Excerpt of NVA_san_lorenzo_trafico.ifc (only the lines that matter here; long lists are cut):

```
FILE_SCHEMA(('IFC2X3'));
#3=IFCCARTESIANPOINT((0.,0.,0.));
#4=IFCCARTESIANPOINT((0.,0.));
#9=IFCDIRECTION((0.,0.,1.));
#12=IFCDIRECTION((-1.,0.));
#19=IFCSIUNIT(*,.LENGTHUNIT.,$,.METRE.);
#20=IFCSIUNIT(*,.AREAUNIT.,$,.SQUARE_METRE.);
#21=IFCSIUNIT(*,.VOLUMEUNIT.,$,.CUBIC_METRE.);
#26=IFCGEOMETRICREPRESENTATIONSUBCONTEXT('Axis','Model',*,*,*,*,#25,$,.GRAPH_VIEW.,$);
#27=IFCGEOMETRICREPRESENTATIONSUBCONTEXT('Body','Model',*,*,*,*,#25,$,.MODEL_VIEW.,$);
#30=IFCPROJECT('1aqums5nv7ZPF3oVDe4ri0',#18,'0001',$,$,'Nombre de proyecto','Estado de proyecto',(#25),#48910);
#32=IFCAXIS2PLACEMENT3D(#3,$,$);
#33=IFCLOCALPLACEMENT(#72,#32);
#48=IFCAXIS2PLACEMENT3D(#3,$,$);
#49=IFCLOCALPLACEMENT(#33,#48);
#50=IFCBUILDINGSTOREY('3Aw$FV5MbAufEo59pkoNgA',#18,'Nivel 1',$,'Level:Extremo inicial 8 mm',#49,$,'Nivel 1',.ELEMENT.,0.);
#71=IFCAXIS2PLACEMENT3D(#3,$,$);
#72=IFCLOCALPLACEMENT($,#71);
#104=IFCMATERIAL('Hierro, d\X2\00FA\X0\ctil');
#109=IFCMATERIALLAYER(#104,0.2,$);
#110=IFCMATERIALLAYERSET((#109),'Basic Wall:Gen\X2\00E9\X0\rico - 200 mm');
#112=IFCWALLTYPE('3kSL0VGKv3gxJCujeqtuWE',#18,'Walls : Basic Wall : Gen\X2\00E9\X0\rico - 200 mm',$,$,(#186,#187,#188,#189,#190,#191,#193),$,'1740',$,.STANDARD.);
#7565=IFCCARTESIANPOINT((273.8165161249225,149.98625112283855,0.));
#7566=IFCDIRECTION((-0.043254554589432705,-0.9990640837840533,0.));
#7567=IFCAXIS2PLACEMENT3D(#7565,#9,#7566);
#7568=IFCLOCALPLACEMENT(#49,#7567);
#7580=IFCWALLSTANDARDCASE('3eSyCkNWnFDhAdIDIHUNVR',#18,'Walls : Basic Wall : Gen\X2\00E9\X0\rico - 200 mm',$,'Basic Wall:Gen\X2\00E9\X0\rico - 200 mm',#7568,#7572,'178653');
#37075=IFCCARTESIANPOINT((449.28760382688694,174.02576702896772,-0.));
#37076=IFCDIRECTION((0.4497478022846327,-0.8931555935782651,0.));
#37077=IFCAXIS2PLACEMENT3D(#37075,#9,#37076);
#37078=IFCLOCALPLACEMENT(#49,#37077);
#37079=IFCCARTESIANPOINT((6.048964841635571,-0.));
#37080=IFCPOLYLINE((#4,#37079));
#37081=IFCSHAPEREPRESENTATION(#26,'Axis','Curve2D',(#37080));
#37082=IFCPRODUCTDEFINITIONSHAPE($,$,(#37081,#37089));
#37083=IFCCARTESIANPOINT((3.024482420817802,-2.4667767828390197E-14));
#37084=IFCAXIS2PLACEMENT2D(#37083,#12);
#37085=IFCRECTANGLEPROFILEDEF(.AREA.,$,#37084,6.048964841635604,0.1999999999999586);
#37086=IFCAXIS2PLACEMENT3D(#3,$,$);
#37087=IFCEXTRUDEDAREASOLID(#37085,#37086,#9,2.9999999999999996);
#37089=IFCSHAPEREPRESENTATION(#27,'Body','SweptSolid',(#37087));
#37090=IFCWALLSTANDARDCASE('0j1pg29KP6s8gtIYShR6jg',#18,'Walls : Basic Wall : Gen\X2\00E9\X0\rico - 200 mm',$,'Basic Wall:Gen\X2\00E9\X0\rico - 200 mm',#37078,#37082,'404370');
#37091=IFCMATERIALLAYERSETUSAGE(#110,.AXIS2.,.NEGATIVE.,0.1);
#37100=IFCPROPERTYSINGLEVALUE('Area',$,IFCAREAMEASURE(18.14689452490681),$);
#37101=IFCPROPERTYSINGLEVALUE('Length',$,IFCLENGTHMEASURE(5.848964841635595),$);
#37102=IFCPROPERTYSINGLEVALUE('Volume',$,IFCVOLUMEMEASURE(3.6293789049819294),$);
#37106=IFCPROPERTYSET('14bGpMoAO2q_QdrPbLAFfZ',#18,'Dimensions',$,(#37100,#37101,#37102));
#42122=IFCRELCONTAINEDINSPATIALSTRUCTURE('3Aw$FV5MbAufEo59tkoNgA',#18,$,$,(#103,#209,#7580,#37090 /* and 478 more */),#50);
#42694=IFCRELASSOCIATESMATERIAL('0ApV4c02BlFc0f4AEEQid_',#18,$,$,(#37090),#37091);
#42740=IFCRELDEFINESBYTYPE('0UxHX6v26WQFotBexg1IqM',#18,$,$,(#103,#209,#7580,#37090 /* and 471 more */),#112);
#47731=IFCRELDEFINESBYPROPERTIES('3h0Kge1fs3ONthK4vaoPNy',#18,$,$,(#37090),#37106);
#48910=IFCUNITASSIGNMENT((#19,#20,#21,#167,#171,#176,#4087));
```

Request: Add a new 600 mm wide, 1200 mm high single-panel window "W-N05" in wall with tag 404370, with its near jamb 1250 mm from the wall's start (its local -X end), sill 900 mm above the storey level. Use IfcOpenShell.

```python
import numpy as np
import ifcopenshell
import ifcopenshell.api.feature
import ifcopenshell.api.geometry
import ifcopenshell.api.pset
import ifcopenshell.api.root
import ifcopenshell.api.spatial
import ifcopenshell.api.type
import ifcopenshell.geom
import ifcopenshell.util.element
import ifcopenshell.util.placement
import ifcopenshell.util.representation
import ifcopenshell.util.shape
import ifcopenshell.util.unit

model = ifcopenshell.open("NVA_san_lorenzo_trafico.ifc")
unit_scale = ifcopenshell.util.unit.calculate_unit_scale(model)
area_scale = ifcopenshell.util.unit.calculate_unit_scale(model, "AREAUNIT")
volume_scale = ifcopenshell.util.unit.calculate_unit_scale(model, "VOLUMEUNIT")
settings = ifcopenshell.geom.settings()


def volume(element):
    """Net volume in cubic metres, openings subtracted."""
    shape = ifcopenshell.geom.create_shape(settings, element)
    return ifcopenshell.util.shape.get_volume(shape.geometry)


wall = model.by_guid("0j1pg29KP6s8gtIYShR6jg")
storey = ifcopenshell.util.element.get_container(wall, ifc_class="IfcBuildingStorey")
context = ifcopenshell.util.representation.get_context(model, "Model", "Body", "MODEL_VIEW")
before = volume(wall)

width, height, from_end, sill = 0.6, 1.2, 1.25, 0.9  # metres

# The wall runs along its own X axis, and the end named is its -X end.
wall_shape = ifcopenshell.geom.create_shape(settings, wall)
x, y, z = ifcopenshell.util.shape.get_vertices(wall_shape.geometry).T
start = x.min() + from_end
face, thickness = float(y.min()), float(y.max() - y.min())
wall_matrix = ifcopenshell.util.placement.get_local_placement(wall.ObjectPlacement)
level = ifcopenshell.util.placement.get_local_placement(storey.ObjectPlacement)[2, 3]


def in_wall(x, y):
    """Placement at x, y metres in the wall's axes, at sill height."""
    matrix = wall_matrix.copy()
    matrix[:, 3] = wall_matrix @ np.array([x / unit_scale, y / unit_scale, 0.0, 1.0])
    matrix[2, 3] = level + sill / unit_scale
    return matrix


# Opening: a box that overshoots both wall faces by 50 mm.
opening = ifcopenshell.api.root.create_entity(model, ifc_class="IfcOpeningElement")
box = ifcopenshell.api.geometry.add_wall_representation(
    model, context=context, length=width, height=height, thickness=thickness + 0.1
)
ifcopenshell.api.geometry.assign_representation(model, product=opening, representation=box)
ifcopenshell.api.geometry.edit_object_placement(model, product=opening, matrix=in_wall(start, face - 0.05), is_si=False)
ifcopenshell.api.feature.add_feature(model, feature=opening, element=wall)

window = ifcopenshell.api.root.create_entity(model, ifc_class="IfcWindow", name="W-N05")
window.OverallWidth, window.OverallHeight = width / unit_scale, height / unit_scale
body = ifcopenshell.api.geometry.add_window_representation(
    model,
    context=context,
    overall_width=window.OverallWidth,
    overall_height=window.OverallHeight,
    partition_type="SINGLE_PANEL",
)
ifcopenshell.api.geometry.assign_representation(model, product=window, representation=body)
ifcopenshell.api.spatial.assign_container(model, products=[window], relating_structure=storey)
fills = ifcopenshell.api.feature.add_filling(model, opening=opening, element=window)
fills.OwnerHistory = window.OwnerHistory  # required in IFC2X3

# IFC2X3 keeps the operation on the window style.
style = ifcopenshell.api.root.create_entity(model, ifc_class="IfcWindowStyle", name="W-N05")
style.OperationType, style.ConstructionType = "SINGLE_PANEL", "NOTDEFINED"
style.ParameterTakesPrecedence = style.Sizeable = False
ifcopenshell.api.type.assign_type(model, related_objects=[window], relating_type=style)

# Centre the window in the wall's thickness.
ifcopenshell.api.geometry.edit_object_placement(model, product=window, matrix=in_wall(start, face), is_si=False)
window_shape = ifcopenshell.geom.create_shape(settings, window)
depth = ifcopenshell.util.shape.get_vertices(window_shape.geometry)[:, 1]
offset = face + thickness / 2 - (depth.min() + depth.max()) / 2
ifcopenshell.api.geometry.edit_object_placement(model, product=window, matrix=in_wall(start, offset), is_si=False)

after = volume(wall)

# Update the wall's stored quantities.
pset = model.by_id(ifcopenshell.util.element.get_pset(wall, "Dimensions", should_inherit=False)["id"])
ifcopenshell.api.pset.edit_pset(model, pset=pset, properties={
    "Area": model.create_entity("IfcAreaMeasure", after / thickness / area_scale),
    "Volume": model.create_entity("IfcVolumeMeasure", after / volume_scale),
})

print(f"wall volume {before:.3f} -> {after:.3f} m3")

model.write("NVA_san_lorenzo_trafico_v2.ifc")
```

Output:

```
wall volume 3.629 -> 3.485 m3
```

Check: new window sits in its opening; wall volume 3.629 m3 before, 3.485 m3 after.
